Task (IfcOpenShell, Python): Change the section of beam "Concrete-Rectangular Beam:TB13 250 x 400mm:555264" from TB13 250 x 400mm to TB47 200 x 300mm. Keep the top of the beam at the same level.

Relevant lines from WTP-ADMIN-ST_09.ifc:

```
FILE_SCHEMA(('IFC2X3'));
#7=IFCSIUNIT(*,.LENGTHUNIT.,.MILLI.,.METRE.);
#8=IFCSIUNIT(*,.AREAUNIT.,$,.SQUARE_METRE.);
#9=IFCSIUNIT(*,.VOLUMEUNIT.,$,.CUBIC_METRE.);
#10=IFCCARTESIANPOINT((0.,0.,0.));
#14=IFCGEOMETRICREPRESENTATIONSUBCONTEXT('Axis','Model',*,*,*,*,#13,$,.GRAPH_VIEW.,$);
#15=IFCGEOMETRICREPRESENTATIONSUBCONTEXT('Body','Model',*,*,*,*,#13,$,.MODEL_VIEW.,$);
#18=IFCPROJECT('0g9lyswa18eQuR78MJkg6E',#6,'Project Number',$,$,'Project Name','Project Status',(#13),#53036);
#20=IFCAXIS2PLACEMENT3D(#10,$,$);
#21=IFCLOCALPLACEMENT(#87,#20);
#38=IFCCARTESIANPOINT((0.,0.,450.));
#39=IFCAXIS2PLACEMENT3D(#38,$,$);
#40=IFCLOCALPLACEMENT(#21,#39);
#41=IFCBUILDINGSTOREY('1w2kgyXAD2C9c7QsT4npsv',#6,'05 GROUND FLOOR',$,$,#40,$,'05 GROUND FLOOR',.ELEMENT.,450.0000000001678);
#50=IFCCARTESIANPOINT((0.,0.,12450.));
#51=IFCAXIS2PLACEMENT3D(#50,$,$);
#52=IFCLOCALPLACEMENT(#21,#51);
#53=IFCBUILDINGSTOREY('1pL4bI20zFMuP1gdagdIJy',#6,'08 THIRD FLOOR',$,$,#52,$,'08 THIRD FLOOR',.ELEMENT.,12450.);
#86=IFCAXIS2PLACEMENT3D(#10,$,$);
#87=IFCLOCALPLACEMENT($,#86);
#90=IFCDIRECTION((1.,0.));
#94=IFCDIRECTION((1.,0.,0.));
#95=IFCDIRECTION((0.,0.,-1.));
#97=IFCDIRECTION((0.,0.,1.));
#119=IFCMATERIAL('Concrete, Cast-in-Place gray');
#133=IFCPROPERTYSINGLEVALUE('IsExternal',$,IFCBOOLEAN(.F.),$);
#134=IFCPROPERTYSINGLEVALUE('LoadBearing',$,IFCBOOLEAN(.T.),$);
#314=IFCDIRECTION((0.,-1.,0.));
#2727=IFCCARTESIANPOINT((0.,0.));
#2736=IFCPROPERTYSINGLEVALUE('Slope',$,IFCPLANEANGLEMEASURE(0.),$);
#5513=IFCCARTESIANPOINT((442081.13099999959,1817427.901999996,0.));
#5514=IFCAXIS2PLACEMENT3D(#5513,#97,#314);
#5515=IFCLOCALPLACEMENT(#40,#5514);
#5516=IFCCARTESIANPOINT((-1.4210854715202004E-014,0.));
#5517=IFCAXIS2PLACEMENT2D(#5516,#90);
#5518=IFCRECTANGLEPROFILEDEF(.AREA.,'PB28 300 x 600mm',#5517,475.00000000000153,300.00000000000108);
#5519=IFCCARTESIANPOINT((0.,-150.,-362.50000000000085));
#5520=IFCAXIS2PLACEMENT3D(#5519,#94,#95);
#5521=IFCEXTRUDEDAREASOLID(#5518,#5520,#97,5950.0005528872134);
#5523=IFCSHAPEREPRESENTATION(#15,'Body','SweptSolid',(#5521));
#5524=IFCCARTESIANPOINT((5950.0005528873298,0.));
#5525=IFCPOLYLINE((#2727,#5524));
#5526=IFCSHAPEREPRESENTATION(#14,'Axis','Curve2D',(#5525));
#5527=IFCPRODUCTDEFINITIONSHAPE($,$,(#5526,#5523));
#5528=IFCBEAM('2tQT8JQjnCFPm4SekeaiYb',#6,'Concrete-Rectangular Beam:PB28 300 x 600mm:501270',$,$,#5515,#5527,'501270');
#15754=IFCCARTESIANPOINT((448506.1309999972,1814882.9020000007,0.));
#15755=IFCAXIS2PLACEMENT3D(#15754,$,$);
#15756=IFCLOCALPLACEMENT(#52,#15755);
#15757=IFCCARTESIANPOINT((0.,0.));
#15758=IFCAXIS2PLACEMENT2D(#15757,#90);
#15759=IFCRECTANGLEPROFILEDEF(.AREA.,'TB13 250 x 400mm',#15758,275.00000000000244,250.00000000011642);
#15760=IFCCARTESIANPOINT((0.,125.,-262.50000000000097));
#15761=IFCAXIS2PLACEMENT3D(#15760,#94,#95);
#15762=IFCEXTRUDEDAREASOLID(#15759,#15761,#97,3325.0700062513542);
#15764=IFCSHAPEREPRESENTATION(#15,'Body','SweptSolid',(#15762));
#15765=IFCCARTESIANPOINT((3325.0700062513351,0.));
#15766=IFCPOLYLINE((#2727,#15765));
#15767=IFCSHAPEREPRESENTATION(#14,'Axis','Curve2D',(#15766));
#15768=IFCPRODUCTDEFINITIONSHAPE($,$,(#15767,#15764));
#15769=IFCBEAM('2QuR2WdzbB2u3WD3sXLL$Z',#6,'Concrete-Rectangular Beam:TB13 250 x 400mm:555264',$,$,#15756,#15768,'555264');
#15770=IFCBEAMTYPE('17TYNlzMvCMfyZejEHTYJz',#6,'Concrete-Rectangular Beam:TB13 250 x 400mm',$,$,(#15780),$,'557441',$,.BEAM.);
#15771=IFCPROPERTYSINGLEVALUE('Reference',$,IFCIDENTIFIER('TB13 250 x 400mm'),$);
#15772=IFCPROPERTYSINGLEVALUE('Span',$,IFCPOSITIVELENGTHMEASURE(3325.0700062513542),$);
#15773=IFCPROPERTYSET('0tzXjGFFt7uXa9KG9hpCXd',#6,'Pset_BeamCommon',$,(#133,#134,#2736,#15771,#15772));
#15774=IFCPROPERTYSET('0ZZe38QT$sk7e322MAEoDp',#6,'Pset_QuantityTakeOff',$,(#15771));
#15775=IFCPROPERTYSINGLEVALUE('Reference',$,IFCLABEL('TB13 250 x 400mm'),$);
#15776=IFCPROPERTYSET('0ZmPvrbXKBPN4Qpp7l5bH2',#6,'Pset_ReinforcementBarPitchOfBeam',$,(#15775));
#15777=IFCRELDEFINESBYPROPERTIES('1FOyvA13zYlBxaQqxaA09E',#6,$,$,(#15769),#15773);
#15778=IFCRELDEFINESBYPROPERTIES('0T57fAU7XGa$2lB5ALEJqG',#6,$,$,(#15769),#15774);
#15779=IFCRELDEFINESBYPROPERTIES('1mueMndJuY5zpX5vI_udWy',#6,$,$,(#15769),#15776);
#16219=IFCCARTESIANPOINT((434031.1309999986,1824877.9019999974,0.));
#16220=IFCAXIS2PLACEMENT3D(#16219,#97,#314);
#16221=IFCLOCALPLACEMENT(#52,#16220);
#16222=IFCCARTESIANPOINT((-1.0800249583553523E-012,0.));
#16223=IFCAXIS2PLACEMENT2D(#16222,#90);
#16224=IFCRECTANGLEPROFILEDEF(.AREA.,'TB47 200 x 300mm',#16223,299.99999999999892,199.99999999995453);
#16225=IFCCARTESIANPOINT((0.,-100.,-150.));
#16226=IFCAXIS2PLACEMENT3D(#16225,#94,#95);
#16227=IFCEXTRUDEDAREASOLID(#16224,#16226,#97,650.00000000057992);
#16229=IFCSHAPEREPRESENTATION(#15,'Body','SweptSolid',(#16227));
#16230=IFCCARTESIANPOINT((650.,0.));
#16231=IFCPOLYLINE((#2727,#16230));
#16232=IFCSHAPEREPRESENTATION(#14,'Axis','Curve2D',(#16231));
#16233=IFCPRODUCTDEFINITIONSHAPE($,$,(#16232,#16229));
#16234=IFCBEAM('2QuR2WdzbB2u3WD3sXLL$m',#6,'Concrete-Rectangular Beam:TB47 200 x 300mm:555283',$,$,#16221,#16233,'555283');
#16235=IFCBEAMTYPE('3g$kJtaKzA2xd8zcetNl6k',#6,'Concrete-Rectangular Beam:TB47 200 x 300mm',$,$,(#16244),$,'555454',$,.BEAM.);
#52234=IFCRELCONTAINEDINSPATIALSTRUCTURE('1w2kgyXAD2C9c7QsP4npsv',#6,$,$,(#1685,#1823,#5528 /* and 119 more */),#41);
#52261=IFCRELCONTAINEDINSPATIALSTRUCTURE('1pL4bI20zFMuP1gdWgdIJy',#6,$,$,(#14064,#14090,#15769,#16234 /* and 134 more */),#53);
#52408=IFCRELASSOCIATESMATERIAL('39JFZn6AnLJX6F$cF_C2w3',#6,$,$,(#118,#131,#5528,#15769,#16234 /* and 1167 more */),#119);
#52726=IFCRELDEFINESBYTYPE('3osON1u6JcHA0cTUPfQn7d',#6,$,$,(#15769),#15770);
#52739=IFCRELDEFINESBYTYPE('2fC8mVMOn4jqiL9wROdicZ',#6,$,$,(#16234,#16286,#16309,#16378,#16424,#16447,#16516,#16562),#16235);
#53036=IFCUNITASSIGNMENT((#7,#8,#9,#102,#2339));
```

```python
import ifcopenshell
import ifcopenshell.api.pset
import ifcopenshell.api.type
import ifcopenshell.util.element
import ifcopenshell.util.representation

model = ifcopenshell.open("WTP-ADMIN-ST_09.ifc")

member = model.by_guid("2QuR2WdzbB2u3WD3sXLL$Z")
source = next(p for p in model.by_type("IfcRectangleProfileDef") if p.ProfileName == "TB47 200 x 300mm")

body = ifcopenshell.util.representation.get_representation(member, "Model", "Body")
solid = body.Items[0]
old_profile = solid.SweptArea

# Copy the section's sizes but keep this member's own profile position.
profile = ifcopenshell.util.element.copy(model, source)
# Profiles are centred, so shift by half the change in depth to hold the top.
shift = (old_profile.XDim - profile.XDim) / 2
x, y = old_profile.Position.Location.Coordinates
up = (-1.0, 0.0)  # upwards, in the solid's own plane
location = model.createIfcCartesianPoint((x + up[0] * shift, y + up[1] * shift))
profile.Position = model.createIfcAxis2Placement2D(location, old_profile.Position.RefDirection)
solid.SweptArea = profile
if not model.get_total_inverses(old_profile):
    ifcopenshell.util.element.remove_deep2(model, old_profile)

new_type = model.by_guid("3g$kJtaKzA2xd8zcetNl6k")
ifcopenshell.api.type.assign_type(
    model, related_objects=[member], relating_type=new_type, should_map_representations=False
)
member.Name = member.Name.replace("TB13 250 x 400mm", "TB47 200 x 300mm")
pset = model.by_id(ifcopenshell.util.element.get_pset(member, "Pset_BeamCommon", should_inherit=False)["id"])
ifcopenshell.api.pset.edit_pset(model, pset=pset, properties={"Reference": "TB47 200 x 300mm"})
pset = model.by_id(ifcopenshell.util.element.get_pset(member, "Pset_QuantityTakeOff", should_inherit=False)["id"])
ifcopenshell.api.pset.edit_pset(model, pset=pset, properties={"Reference": "TB47 200 x 300mm"})
pset = model.by_id(ifcopenshell.util.element.get_pset(member, "Pset_ReinforcementBarPitchOfBeam", should_inherit=False)["id"])
ifcopenshell.api.pset.edit_pset(model, pset=pset, properties={"Reference": "TB47 200 x 300mm"})

print(solid.SweptArea)

model.write("WTP-ADMIN-ST_09_rev.ifc")
```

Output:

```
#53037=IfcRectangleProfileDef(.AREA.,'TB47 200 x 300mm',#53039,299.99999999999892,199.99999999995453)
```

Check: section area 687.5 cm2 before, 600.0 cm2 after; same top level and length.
